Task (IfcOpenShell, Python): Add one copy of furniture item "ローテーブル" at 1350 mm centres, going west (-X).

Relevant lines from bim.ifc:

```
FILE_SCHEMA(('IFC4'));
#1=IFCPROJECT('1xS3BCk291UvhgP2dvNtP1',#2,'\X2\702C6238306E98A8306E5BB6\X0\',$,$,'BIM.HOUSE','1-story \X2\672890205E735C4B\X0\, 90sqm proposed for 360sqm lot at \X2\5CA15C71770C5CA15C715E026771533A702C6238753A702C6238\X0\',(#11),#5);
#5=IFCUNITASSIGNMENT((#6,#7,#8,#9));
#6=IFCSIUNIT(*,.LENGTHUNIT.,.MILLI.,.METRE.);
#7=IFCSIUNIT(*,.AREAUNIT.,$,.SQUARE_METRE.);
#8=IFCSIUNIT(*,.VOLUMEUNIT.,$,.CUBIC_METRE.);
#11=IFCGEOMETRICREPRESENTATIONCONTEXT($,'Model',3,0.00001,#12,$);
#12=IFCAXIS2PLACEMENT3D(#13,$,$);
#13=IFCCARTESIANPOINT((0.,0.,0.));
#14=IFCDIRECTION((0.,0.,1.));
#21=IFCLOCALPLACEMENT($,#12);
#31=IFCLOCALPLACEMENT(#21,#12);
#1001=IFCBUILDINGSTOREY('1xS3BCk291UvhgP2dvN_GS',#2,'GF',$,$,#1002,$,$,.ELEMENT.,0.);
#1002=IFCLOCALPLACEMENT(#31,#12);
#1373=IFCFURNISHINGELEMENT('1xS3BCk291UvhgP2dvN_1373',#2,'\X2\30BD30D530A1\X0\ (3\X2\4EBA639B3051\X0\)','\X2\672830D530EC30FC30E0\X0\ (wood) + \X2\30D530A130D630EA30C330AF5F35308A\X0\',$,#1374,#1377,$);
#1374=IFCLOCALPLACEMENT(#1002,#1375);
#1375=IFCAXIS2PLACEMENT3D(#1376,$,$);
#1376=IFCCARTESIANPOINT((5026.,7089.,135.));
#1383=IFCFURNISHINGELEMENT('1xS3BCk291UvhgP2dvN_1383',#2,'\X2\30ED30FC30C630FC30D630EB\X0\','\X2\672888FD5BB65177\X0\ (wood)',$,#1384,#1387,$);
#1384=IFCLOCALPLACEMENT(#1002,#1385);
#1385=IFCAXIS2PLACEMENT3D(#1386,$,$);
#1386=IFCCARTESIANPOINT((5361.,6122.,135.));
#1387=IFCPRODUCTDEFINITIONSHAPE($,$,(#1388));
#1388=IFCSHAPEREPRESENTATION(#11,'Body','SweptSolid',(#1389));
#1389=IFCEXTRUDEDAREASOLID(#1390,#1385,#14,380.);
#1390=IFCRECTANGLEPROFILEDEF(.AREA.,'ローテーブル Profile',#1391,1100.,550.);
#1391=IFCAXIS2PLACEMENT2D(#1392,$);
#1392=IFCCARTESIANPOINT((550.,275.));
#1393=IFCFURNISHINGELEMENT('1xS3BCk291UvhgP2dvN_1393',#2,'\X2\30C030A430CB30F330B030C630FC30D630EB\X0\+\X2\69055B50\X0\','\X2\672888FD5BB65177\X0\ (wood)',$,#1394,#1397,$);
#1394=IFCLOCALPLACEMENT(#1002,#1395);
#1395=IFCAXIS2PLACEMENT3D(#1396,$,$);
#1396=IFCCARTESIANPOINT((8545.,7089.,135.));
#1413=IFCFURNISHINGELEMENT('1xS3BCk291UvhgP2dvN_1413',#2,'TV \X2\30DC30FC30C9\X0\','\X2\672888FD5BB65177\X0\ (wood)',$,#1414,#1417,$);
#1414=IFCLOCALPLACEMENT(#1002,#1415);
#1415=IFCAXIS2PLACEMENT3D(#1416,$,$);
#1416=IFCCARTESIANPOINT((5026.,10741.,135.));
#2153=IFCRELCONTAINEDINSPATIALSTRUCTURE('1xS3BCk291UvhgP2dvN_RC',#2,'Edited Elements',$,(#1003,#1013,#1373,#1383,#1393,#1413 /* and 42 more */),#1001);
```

```python
import numpy as np
import ifcopenshell
import ifcopenshell.api.geometry
import ifcopenshell.api.root
import ifcopenshell.util.element
import ifcopenshell.util.placement
import ifcopenshell.util.unit

model = ifcopenshell.open("bim.ifc")
unit_scale = ifcopenshell.util.unit.calculate_unit_scale(model)


def reuse_history(source, copy):
    """copy_class also copies each property set's owner history, people and application; keep the originals."""
    for rel in copy.IsDefinedBy:
        if rel.is_a("IfcRelDefinesByProperties") and (history := rel.RelatingPropertyDefinition.OwnerHistory):
            rel.RelatingPropertyDefinition.OwnerHistory = source.OwnerHistory
            ifcopenshell.util.element.remove_deep2(model, history)


source = model.by_guid("1xS3BCk291UvhgP2dvN_1383")
base = ifcopenshell.util.placement.get_local_placement(source.ObjectPlacement)
step = np.array([-1.0, 0.0, 0.0]) * 1.35 / unit_scale

for i in range(1, 2):
    copy = ifcopenshell.api.root.copy_class(model, product=source)
    copy.Representation = ifcopenshell.util.element.copy_deep(
        model, source.Representation, exclude=["IfcGeometricRepresentationContext", "IfcRepresentationMap"]
    )
    reuse_history(source, copy)
    matrix = base.copy()
    matrix[:3, 3] += i * step
    print("added at", matrix[:3, 3].round(3) + 0.0)
    ifcopenshell.api.geometry.edit_object_placement(model, product=copy, matrix=matrix, is_si=False)

model.write("bim_rev.ifc")
```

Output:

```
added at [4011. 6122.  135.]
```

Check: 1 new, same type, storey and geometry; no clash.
